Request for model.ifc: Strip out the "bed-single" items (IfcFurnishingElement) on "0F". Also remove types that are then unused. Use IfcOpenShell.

First a look at what the model holds.

```python
import ifcopenshell
import ifcopenshell.util.element

model = ifcopenshell.open("model.ifc")
print(model.schema)
storey = next(s for s in model.by_type("IfcBuildingStorey") if s.Name == "0F")
furniture = [e for e in ifcopenshell.util.element.get_decomposition(storey) if e.is_a("IfcFurnishingElement")]
seen = {}
for e in furniture:
    element_type = ifcopenshell.util.element.get_type(e)
    name = element_type.Name if element_type not in (None, e) else None
    seen[name] = seen.get(name, 0) + 1
for name, count in sorted(seen.items(), key=str):
    print(count, "x", name)
```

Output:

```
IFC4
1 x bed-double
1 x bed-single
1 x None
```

```python
import ifcopenshell
import ifcopenshell.api.root
import ifcopenshell.util.element

model = ifcopenshell.open("model.ifc")

storey = next(s for s in model.by_type("IfcBuildingStorey") if s.Name == "0F")
furniture = [e for e in ifcopenshell.util.element.get_decomposition(storey) if e.is_a("IfcFurnishingElement")]
targets = [e for e in furniture if (t := ifcopenshell.util.element.get_type(e)) not in (None, e) and t.Name == "bed-single"]
types = {ifcopenshell.util.element.get_type(e) for e in targets} - {None, *targets}

for e in targets:
    ifcopenshell.api.root.remove_product(model, product=e)
print(len(targets), "removed")

unused = [t for t in types if not ifcopenshell.util.element.get_types(t)]
for t in unused:
    ifcopenshell.api.root.remove_product(model, product=t)
print(len(unused), "unused types removed")

model.write("model_edited.ifc")
```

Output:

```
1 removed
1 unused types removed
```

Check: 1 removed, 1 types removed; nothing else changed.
